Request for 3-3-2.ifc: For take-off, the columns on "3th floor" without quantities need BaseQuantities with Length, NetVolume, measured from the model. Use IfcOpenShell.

First a look at what the model holds.

```python
import ifcopenshell
import ifcopenshell.util.element
import ifcopenshell.util.unit

model = ifcopenshell.open("3-3-2.ifc")
print(model.schema)
for unit_type in ("LENGTHUNIT", "AREAUNIT", "VOLUMEUNIT"):
    print(unit_type, ifcopenshell.util.unit.calculate_unit_scale(model, unit_type))
storey = next(s for s in model.by_type("IfcBuildingStorey") if s.Name == "3th floor")
columns = [e for e in ifcopenshell.util.element.get_decomposition(storey) if e.is_a("IfcColumn")]
for e in sorted(columns, key=lambda e: e.id()):
    print(e.id(), e.is_a(), e.Name, list(ifcopenshell.util.element.get_psets(e, qtos_only=True)), sep=" | ")
```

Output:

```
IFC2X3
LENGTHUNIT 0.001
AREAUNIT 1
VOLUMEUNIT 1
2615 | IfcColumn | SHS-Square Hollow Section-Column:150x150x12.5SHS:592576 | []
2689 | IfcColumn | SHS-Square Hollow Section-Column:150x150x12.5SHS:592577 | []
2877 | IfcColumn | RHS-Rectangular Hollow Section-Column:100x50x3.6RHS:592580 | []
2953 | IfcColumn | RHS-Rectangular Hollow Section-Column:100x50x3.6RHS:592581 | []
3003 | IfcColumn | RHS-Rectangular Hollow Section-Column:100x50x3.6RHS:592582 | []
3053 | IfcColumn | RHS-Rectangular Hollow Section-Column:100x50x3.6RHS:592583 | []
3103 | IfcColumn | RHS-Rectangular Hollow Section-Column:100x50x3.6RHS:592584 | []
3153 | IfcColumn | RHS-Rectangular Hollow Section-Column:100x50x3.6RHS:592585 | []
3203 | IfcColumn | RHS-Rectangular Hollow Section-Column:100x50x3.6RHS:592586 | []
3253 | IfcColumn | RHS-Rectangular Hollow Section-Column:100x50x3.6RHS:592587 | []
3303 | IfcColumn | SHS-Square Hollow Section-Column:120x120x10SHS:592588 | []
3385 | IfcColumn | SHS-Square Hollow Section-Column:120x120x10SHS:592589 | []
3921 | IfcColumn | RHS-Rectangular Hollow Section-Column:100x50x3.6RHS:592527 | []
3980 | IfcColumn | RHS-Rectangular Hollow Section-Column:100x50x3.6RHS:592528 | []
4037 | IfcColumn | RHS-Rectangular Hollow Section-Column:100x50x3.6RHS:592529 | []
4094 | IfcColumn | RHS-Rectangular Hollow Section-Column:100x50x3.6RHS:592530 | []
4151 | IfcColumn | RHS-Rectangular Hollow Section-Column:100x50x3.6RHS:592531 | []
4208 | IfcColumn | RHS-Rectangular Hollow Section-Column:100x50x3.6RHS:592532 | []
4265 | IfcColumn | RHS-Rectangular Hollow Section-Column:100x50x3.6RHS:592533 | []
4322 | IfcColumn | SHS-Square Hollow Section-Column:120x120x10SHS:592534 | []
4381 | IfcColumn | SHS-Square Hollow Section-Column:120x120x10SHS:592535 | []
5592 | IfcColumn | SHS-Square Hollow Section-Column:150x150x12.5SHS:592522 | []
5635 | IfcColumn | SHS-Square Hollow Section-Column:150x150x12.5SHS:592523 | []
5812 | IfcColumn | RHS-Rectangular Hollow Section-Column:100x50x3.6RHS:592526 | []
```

```python
import ifcopenshell
import ifcopenshell.api.pset
import ifcopenshell.geom
import ifcopenshell.util.element
import ifcopenshell.util.shape
import ifcopenshell.util.unit

model = ifcopenshell.open("3-3-2.ifc")
unit_scale = ifcopenshell.util.unit.calculate_unit_scale(model)
volume_scale = ifcopenshell.util.unit.calculate_unit_scale(model, "VOLUMEUNIT")
settings = ifcopenshell.geom.settings()

storey = next(s for s in model.by_type("IfcBuildingStorey") if s.Name == "3th floor")
columns = [e for e in ifcopenshell.util.element.get_decomposition(storey) if e.is_a("IfcColumn")]

for e in sorted(columns, key=lambda e: e.id()):
    if ifcopenshell.util.element.get_psets(e, qtos_only=True, should_inherit=False):
        continue
    # Geometry comes back in metres, in the element's own axes.
    shape = ifcopenshell.geom.create_shape(settings, e)
    values = {
        "Length": ifcopenshell.util.shape.get_z(shape.geometry) / unit_scale,
        "NetVolume": ifcopenshell.util.shape.get_volume(shape.geometry) / volume_scale,
    }
    qto = ifcopenshell.api.pset.add_qto(model, product=e, name="BaseQuantities")
    ifcopenshell.api.pset.edit_qto(model, qto=qto, properties=values)
    print(e.id(), {k: round(v, 3) for k, v in values.items()})

model.write("3-3-2_rev.ifc")
```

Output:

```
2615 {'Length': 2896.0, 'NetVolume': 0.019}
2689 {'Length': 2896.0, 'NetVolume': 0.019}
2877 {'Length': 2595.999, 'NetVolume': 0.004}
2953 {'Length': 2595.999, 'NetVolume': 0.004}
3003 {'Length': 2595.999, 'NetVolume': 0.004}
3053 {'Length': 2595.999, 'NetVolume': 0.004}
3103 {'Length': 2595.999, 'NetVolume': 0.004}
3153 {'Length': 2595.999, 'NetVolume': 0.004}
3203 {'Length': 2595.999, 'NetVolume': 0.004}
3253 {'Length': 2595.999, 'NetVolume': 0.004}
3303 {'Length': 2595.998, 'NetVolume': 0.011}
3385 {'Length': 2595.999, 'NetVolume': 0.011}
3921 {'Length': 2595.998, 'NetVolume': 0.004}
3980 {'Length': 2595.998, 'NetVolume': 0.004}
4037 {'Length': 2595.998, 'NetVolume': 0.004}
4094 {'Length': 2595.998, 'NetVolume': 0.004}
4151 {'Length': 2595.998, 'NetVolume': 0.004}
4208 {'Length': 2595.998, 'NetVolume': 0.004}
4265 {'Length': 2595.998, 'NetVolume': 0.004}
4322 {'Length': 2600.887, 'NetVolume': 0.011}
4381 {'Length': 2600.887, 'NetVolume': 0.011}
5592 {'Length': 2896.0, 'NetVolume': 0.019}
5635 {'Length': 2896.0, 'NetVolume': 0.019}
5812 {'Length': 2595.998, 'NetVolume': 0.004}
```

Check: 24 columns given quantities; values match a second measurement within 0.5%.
